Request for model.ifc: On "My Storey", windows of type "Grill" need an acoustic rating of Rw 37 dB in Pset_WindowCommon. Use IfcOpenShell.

First a look at what the model holds.

```python
import ifcopenshell
import ifcopenshell.util.element

model = ifcopenshell.open("model.ifc")
print(model.schema)
storey = next(s for s in model.by_type("IfcBuildingStorey") if s.Name == "My Storey")
windows = [e for e in ifcopenshell.util.element.get_decomposition(storey) if e.is_a("IfcWindow")]
seen = {}
for e in windows:
    element_type = ifcopenshell.util.element.get_type(e)
    key = (element_type.Name if element_type != e and element_type else None, ifcopenshell.util.element.get_pset(e, "Pset_WindowCommon", "AcousticRating"))
    seen[key] = seen.get(key, 0) + 1
for (name, value), count in sorted(seen.items(), key=str):
    print(count, "x", name, "|", value)
```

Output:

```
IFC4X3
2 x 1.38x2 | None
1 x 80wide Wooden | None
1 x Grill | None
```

```python
import ifcopenshell
import ifcopenshell.api.pset
import ifcopenshell.util.element

model = ifcopenshell.open("model.ifc")

storey = next(s for s in model.by_type("IfcBuildingStorey") if s.Name == "My Storey")
windows = [e for e in ifcopenshell.util.element.get_decomposition(storey) if e.is_a("IfcWindow")]

count = 0
for e in windows:
    element_type = ifcopenshell.util.element.get_type(e)
    if element_type in (None, e) or element_type.Name != "Grill":
        continue
    # add_pset returns the element's existing set when there is one.
    pset = ifcopenshell.api.pset.add_pset(model, product=e, name="Pset_WindowCommon")
    ifcopenshell.api.pset.edit_pset(model, pset=pset, properties={"AcousticRating": "Rw 37 dB"})
    count += 1

print(count, "windows updated")

model.write("model_edited.ifc")
```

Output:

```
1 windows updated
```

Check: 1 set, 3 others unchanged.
